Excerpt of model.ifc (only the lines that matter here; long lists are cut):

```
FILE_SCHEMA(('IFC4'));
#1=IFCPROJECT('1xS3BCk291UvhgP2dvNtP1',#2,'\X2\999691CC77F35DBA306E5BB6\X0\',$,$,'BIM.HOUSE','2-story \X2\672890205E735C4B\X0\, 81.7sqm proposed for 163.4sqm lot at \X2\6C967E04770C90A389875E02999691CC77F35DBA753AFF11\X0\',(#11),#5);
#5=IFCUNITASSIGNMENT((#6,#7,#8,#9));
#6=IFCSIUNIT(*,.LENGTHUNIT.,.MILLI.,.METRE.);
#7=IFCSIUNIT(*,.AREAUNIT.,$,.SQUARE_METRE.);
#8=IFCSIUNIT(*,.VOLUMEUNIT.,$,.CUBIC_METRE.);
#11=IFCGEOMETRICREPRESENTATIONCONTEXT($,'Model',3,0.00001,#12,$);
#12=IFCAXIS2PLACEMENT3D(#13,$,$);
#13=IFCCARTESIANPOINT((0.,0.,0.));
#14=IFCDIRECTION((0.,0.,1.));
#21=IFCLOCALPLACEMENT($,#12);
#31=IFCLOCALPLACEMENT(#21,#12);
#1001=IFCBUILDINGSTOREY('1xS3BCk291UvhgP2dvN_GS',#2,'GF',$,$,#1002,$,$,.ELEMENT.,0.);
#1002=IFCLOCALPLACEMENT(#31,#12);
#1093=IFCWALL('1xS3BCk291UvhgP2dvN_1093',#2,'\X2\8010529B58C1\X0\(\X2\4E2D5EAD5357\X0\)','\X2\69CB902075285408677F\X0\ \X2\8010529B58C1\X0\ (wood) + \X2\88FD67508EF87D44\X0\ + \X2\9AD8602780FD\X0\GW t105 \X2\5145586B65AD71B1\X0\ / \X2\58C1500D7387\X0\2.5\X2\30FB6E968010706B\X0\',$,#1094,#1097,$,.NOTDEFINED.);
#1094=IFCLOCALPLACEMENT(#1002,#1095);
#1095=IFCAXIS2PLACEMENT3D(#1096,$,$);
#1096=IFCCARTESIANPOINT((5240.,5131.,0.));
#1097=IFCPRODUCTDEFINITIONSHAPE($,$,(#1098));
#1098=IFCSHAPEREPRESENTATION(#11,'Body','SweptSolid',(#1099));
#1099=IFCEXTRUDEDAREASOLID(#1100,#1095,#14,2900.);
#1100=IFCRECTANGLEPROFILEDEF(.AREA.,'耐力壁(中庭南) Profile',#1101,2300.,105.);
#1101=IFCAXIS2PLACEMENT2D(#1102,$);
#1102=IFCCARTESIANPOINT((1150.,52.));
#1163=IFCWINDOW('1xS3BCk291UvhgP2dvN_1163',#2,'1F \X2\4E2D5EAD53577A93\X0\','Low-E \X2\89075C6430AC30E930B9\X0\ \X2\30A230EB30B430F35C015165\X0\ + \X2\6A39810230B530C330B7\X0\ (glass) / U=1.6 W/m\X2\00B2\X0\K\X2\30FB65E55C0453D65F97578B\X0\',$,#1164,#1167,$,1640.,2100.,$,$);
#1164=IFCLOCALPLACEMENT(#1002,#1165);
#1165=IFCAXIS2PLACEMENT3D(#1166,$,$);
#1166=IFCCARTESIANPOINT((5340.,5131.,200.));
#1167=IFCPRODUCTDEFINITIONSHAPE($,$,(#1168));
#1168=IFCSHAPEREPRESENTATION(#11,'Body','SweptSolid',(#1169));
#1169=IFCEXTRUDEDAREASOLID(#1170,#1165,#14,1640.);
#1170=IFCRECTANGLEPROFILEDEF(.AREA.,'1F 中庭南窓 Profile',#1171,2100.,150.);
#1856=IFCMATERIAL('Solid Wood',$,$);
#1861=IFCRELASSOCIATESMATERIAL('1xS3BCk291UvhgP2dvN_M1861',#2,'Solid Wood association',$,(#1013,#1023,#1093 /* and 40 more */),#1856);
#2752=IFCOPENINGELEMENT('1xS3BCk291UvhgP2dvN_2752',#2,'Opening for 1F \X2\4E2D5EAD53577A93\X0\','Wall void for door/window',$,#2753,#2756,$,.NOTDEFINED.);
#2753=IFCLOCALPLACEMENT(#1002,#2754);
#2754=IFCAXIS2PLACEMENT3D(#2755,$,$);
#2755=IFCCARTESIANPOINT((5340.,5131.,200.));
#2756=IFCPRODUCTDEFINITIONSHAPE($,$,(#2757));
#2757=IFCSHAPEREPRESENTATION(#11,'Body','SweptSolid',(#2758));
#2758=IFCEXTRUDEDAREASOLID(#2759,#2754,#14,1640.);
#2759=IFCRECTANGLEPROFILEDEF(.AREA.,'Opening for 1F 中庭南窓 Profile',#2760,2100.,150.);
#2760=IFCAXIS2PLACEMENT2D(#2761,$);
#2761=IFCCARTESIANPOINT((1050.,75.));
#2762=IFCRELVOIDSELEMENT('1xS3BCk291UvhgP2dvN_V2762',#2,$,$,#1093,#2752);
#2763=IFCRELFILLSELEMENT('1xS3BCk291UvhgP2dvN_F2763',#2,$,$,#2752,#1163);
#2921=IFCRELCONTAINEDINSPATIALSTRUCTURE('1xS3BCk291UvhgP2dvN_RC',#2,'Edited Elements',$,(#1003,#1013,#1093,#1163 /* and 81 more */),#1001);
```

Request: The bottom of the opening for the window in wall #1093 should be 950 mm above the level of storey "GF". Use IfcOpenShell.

```python
import numpy as np
import ifcopenshell
import ifcopenshell.api.geometry
import ifcopenshell.geom
import ifcopenshell.util.element
import ifcopenshell.util.placement
import ifcopenshell.util.shape
import ifcopenshell.util.unit

model = ifcopenshell.open("model.ifc")
unit_scale = ifcopenshell.util.unit.calculate_unit_scale(model)

window = model.by_guid("1xS3BCk291UvhgP2dvN_1163")
opening = window.FillsVoids[0].RelatingOpeningElement
storey = ifcopenshell.util.element.get_container(window, ifc_class="IfcBuildingStorey")
level = ifcopenshell.util.placement.get_local_placement(storey.ObjectPlacement)[2, 3]

# The opening's origin need not be at the sill, so measure its lowest point.
shape = ifcopenshell.geom.create_shape(ifcopenshell.geom.settings(), opening)
bottom = ifcopenshell.util.shape.get_shape_bottom_elevation(shape, shape.geometry) / unit_scale
dz = level + 0.95 / unit_scale - bottom

shift = np.array([0.0, 0.0, dz])
# The window is not placed relative to its opening, so move both.
for product in (opening, window):
    matrix = ifcopenshell.util.placement.get_local_placement(product.ObjectPlacement)
    matrix[:3, 3] += shift
    ifcopenshell.api.geometry.edit_object_placement(model, product=product, matrix=matrix, is_si=False)

print(f"moved by {dz * unit_scale:+.3f} m")

model.write("model_updated.ifc")
```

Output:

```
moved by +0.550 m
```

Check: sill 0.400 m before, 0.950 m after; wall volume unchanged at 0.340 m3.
